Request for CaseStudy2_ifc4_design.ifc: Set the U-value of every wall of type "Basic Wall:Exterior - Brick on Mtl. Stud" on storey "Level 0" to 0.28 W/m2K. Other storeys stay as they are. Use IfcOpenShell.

First a look at what the model holds.

```python
import ifcopenshell
import ifcopenshell.util.element

model = ifcopenshell.open("CaseStudy2_ifc4_design.ifc")
print(model.schema)
storey = next(s for s in model.by_type("IfcBuildingStorey") if s.Name == "Level 0")
walls = [e for e in ifcopenshell.util.element.get_decomposition(storey) if e.is_a("IfcWall")]
seen = {}
for e in walls:
    element_type = ifcopenshell.util.element.get_type(e)
    key = (element_type.Name if element_type != e and element_type else None, ifcopenshell.util.element.get_pset(e, "Pset_WallCommon", "ThermalTransmittance"))
    seen[key] = seen.get(key, 0) + 1
for (name, value), count in sorted(seen.items(), key=str):
    print(count, "x", name, "|", value)
```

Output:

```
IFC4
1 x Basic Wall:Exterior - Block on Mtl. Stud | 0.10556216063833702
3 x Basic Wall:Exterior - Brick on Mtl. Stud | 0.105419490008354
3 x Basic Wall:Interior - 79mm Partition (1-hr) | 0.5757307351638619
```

```python
import ifcopenshell
import ifcopenshell.api.pset
import ifcopenshell.util.element

model = ifcopenshell.open("CaseStudy2_ifc4_design.ifc")

storey = next(s for s in model.by_type("IfcBuildingStorey") if s.Name == "Level 0")
walls = [e for e in ifcopenshell.util.element.get_decomposition(storey) if e.is_a("IfcWall")]

count = 0
for e in walls:
    element_type = ifcopenshell.util.element.get_type(e)
    if element_type in (None, e) or element_type.Name != "Basic Wall:Exterior - Brick on Mtl. Stud":
        continue
    # add_pset returns the element's existing set when there is one.
    pset = ifcopenshell.api.pset.add_pset(model, product=e, name="Pset_WallCommon")
    ifcopenshell.api.pset.edit_pset(model, pset=pset, properties={"ThermalTransmittance": 0.28})
    count += 1

print(count, "walls updated")

model.write("CaseStudy2_ifc4_design_updated.ifc")
```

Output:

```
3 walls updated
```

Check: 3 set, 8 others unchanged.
